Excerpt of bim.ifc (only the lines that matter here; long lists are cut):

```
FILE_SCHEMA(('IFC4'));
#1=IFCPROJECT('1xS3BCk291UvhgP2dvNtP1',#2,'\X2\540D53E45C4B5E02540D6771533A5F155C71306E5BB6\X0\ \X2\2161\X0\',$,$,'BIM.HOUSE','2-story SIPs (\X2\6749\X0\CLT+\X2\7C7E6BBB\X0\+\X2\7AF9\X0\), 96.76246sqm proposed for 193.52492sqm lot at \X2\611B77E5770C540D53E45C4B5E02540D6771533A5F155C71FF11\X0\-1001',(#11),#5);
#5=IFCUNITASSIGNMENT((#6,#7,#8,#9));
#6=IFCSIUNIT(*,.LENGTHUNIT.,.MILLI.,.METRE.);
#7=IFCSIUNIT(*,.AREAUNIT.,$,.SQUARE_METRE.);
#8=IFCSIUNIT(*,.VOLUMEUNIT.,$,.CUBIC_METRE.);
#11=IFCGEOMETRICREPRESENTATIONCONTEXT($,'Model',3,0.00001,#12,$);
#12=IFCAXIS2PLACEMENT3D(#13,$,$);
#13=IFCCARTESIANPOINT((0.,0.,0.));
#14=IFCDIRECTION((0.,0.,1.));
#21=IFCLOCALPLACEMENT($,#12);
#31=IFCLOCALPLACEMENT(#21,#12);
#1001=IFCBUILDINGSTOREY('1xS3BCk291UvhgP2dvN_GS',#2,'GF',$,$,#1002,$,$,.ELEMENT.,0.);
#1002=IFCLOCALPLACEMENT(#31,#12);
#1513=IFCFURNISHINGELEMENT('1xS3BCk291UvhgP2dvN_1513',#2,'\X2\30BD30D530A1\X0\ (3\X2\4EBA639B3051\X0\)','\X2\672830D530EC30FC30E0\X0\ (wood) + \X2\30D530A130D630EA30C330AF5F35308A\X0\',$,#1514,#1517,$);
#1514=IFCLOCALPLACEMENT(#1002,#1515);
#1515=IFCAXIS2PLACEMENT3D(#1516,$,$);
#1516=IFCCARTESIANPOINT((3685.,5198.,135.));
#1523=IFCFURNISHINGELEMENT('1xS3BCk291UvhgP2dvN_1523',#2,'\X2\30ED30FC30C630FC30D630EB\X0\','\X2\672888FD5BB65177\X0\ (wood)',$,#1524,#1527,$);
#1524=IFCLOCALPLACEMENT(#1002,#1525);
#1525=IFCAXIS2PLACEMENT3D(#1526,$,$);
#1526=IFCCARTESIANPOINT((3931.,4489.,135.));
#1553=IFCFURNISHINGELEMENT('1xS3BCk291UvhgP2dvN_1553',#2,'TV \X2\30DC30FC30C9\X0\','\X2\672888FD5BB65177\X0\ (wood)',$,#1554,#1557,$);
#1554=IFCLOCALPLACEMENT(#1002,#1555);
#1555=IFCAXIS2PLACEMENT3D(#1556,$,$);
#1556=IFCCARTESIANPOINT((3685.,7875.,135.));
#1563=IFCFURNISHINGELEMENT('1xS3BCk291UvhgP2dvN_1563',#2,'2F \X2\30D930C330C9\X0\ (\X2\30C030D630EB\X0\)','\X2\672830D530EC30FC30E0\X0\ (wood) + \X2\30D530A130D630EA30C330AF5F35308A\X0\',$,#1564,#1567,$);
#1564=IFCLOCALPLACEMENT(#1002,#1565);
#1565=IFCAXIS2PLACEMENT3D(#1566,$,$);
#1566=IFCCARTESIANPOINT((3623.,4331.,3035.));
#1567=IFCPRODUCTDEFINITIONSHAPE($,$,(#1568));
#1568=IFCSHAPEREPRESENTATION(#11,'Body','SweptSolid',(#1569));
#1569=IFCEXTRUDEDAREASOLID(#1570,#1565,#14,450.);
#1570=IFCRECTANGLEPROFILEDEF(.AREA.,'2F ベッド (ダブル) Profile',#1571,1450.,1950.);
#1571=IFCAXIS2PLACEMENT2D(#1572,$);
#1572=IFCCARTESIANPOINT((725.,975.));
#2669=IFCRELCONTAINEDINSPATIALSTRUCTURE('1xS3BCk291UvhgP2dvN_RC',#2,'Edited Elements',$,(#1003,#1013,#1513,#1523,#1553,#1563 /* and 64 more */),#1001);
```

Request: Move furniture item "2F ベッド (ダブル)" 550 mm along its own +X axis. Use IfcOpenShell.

```python
import ifcopenshell
import ifcopenshell.api.geometry
import ifcopenshell.util.placement

model = ifcopenshell.open("bim.ifc")

item = model.by_guid("1xS3BCk291UvhgP2dvN_1563")
matrix = ifcopenshell.util.placement.get_local_placement(item.ObjectPlacement)
matrix[:3, 3] += matrix[:3, 0] * 550.0
ifcopenshell.api.geometry.edit_object_placement(model, product=item, matrix=matrix, is_si=False)

print(ifcopenshell.util.placement.get_local_placement(item.ObjectPlacement).round(3) + 0.0)

model.write("bim-out.ifc")
```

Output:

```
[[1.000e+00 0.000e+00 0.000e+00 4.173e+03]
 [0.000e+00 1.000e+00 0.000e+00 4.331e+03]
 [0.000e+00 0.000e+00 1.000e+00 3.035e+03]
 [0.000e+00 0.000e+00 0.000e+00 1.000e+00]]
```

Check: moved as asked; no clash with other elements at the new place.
